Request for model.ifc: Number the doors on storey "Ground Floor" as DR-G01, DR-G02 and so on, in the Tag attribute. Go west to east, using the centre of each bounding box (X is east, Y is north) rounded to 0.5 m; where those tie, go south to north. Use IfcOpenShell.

First a look at what the model holds.

```python
import ifcopenshell
import ifcopenshell.util.element
import ifcopenshell.util.placement

model = ifcopenshell.open("model.ifc")
print(model.schema)
storey = next(s for s in model.by_type("IfcBuildingStorey") if s.Name == "Ground Floor")
doors = [e for e in ifcopenshell.util.element.get_decomposition(storey) if e.is_a("IfcDoor")]
for e in sorted(doors, key=lambda e: e.id()):
    origin = ifcopenshell.util.placement.get_local_placement(e.ObjectPlacement)[:3, 3]
    print(e.id(), e.Tag, e.Name, origin.round(2) + 0.0, sep=" | ")
```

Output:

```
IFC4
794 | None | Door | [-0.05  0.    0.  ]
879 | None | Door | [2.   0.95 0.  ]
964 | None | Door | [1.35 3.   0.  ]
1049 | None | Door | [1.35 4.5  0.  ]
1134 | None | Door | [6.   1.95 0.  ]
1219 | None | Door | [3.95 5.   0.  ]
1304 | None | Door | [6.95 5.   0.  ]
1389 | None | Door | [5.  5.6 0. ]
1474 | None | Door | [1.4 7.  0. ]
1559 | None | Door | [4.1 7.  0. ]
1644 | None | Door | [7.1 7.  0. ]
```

```python
import ifcopenshell
import ifcopenshell.geom
import ifcopenshell.util.element
import ifcopenshell.util.shape

model = ifcopenshell.open("model.ifc")
settings = ifcopenshell.geom.settings()
settings.set("use-world-coords", True)


def centre(element):
    shape = ifcopenshell.geom.create_shape(settings, element)
    return ifcopenshell.util.shape.get_bbox_centroid(shape.geometry)


storey = next(s for s in model.by_type("IfcBuildingStorey") if s.Name == "Ground Floor")
doors = [e for e in ifcopenshell.util.element.get_decomposition(storey) if e.is_a("IfcDoor")]

# Insertion points can sit at a corner or the storey origin, so sort by the geometry (in metres).
centres = {e: centre(e) for e in doors}
doors.sort(key=lambda e: (round(centres[e][0] / 0.5), centres[e][1]))

for i, e in enumerate(doors, start=1):
    number = f"DR-G{i:02d}"
    e.Tag = number
    print(e.id(), number)

model.write("model_rev.ifc")
```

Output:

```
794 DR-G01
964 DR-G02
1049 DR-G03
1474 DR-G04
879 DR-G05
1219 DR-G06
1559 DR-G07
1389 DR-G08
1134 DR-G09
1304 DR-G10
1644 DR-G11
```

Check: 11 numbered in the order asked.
